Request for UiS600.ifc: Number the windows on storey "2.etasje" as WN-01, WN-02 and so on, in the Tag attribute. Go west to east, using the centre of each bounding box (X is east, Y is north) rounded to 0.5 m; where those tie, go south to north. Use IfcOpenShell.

First a look at what the model holds.

```python
import ifcopenshell
import ifcopenshell.util.element
import ifcopenshell.util.placement

model = ifcopenshell.open("UiS600.ifc")
print(model.schema)
storey = next(s for s in model.by_type("IfcBuildingStorey") if s.Name == "2.etasje")
windows = [e for e in ifcopenshell.util.element.get_decomposition(storey) if e.is_a("IfcWindow")]
for e in sorted(windows, key=lambda e: e.id()):
    origin = ifcopenshell.util.placement.get_local_placement(e.ObjectPlacement)[:3, 3]
    print(e.id(), e.Tag, e.Name, origin.round(2) + 0.0, sep=" | ")
```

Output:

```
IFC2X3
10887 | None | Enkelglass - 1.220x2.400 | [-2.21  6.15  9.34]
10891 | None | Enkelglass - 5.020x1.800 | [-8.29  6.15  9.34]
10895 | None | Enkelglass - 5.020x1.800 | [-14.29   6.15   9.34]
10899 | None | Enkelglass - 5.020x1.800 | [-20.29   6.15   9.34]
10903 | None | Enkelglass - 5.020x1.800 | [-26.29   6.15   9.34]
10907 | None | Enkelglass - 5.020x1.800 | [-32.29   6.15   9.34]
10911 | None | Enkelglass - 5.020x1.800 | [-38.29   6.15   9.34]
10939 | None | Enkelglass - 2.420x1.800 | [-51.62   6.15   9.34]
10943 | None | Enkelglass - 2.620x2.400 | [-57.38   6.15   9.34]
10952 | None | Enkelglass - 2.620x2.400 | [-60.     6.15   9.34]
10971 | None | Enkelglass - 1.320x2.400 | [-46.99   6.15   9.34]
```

```python
import ifcopenshell
import ifcopenshell.geom
import ifcopenshell.util.element
import ifcopenshell.util.shape

model = ifcopenshell.open("UiS600.ifc")
settings = ifcopenshell.geom.settings()
settings.set("use-world-coords", True)


def centre(element):
    shape = ifcopenshell.geom.create_shape(settings, element)
    return ifcopenshell.util.shape.get_bbox_centroid(shape.geometry)


storey = next(s for s in model.by_type("IfcBuildingStorey") if s.Name == "2.etasje")
windows = [e for e in ifcopenshell.util.element.get_decomposition(storey) if e.is_a("IfcWindow")]

# Insertion points can sit at a corner or the storey origin, so sort by the geometry (in metres).
centres = {e: centre(e) for e in windows}
windows.sort(key=lambda e: (round(centres[e][0] / 0.5), centres[e][1]))

for i, e in enumerate(windows, start=1):
    number = f"WN-{i:02d}"
    e.Tag = number
    print(e.id(), number)

model.write("UiS600_rev.ifc")
```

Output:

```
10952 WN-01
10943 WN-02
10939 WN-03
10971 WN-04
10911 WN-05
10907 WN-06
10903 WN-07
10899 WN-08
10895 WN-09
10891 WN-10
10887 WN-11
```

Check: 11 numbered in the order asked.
